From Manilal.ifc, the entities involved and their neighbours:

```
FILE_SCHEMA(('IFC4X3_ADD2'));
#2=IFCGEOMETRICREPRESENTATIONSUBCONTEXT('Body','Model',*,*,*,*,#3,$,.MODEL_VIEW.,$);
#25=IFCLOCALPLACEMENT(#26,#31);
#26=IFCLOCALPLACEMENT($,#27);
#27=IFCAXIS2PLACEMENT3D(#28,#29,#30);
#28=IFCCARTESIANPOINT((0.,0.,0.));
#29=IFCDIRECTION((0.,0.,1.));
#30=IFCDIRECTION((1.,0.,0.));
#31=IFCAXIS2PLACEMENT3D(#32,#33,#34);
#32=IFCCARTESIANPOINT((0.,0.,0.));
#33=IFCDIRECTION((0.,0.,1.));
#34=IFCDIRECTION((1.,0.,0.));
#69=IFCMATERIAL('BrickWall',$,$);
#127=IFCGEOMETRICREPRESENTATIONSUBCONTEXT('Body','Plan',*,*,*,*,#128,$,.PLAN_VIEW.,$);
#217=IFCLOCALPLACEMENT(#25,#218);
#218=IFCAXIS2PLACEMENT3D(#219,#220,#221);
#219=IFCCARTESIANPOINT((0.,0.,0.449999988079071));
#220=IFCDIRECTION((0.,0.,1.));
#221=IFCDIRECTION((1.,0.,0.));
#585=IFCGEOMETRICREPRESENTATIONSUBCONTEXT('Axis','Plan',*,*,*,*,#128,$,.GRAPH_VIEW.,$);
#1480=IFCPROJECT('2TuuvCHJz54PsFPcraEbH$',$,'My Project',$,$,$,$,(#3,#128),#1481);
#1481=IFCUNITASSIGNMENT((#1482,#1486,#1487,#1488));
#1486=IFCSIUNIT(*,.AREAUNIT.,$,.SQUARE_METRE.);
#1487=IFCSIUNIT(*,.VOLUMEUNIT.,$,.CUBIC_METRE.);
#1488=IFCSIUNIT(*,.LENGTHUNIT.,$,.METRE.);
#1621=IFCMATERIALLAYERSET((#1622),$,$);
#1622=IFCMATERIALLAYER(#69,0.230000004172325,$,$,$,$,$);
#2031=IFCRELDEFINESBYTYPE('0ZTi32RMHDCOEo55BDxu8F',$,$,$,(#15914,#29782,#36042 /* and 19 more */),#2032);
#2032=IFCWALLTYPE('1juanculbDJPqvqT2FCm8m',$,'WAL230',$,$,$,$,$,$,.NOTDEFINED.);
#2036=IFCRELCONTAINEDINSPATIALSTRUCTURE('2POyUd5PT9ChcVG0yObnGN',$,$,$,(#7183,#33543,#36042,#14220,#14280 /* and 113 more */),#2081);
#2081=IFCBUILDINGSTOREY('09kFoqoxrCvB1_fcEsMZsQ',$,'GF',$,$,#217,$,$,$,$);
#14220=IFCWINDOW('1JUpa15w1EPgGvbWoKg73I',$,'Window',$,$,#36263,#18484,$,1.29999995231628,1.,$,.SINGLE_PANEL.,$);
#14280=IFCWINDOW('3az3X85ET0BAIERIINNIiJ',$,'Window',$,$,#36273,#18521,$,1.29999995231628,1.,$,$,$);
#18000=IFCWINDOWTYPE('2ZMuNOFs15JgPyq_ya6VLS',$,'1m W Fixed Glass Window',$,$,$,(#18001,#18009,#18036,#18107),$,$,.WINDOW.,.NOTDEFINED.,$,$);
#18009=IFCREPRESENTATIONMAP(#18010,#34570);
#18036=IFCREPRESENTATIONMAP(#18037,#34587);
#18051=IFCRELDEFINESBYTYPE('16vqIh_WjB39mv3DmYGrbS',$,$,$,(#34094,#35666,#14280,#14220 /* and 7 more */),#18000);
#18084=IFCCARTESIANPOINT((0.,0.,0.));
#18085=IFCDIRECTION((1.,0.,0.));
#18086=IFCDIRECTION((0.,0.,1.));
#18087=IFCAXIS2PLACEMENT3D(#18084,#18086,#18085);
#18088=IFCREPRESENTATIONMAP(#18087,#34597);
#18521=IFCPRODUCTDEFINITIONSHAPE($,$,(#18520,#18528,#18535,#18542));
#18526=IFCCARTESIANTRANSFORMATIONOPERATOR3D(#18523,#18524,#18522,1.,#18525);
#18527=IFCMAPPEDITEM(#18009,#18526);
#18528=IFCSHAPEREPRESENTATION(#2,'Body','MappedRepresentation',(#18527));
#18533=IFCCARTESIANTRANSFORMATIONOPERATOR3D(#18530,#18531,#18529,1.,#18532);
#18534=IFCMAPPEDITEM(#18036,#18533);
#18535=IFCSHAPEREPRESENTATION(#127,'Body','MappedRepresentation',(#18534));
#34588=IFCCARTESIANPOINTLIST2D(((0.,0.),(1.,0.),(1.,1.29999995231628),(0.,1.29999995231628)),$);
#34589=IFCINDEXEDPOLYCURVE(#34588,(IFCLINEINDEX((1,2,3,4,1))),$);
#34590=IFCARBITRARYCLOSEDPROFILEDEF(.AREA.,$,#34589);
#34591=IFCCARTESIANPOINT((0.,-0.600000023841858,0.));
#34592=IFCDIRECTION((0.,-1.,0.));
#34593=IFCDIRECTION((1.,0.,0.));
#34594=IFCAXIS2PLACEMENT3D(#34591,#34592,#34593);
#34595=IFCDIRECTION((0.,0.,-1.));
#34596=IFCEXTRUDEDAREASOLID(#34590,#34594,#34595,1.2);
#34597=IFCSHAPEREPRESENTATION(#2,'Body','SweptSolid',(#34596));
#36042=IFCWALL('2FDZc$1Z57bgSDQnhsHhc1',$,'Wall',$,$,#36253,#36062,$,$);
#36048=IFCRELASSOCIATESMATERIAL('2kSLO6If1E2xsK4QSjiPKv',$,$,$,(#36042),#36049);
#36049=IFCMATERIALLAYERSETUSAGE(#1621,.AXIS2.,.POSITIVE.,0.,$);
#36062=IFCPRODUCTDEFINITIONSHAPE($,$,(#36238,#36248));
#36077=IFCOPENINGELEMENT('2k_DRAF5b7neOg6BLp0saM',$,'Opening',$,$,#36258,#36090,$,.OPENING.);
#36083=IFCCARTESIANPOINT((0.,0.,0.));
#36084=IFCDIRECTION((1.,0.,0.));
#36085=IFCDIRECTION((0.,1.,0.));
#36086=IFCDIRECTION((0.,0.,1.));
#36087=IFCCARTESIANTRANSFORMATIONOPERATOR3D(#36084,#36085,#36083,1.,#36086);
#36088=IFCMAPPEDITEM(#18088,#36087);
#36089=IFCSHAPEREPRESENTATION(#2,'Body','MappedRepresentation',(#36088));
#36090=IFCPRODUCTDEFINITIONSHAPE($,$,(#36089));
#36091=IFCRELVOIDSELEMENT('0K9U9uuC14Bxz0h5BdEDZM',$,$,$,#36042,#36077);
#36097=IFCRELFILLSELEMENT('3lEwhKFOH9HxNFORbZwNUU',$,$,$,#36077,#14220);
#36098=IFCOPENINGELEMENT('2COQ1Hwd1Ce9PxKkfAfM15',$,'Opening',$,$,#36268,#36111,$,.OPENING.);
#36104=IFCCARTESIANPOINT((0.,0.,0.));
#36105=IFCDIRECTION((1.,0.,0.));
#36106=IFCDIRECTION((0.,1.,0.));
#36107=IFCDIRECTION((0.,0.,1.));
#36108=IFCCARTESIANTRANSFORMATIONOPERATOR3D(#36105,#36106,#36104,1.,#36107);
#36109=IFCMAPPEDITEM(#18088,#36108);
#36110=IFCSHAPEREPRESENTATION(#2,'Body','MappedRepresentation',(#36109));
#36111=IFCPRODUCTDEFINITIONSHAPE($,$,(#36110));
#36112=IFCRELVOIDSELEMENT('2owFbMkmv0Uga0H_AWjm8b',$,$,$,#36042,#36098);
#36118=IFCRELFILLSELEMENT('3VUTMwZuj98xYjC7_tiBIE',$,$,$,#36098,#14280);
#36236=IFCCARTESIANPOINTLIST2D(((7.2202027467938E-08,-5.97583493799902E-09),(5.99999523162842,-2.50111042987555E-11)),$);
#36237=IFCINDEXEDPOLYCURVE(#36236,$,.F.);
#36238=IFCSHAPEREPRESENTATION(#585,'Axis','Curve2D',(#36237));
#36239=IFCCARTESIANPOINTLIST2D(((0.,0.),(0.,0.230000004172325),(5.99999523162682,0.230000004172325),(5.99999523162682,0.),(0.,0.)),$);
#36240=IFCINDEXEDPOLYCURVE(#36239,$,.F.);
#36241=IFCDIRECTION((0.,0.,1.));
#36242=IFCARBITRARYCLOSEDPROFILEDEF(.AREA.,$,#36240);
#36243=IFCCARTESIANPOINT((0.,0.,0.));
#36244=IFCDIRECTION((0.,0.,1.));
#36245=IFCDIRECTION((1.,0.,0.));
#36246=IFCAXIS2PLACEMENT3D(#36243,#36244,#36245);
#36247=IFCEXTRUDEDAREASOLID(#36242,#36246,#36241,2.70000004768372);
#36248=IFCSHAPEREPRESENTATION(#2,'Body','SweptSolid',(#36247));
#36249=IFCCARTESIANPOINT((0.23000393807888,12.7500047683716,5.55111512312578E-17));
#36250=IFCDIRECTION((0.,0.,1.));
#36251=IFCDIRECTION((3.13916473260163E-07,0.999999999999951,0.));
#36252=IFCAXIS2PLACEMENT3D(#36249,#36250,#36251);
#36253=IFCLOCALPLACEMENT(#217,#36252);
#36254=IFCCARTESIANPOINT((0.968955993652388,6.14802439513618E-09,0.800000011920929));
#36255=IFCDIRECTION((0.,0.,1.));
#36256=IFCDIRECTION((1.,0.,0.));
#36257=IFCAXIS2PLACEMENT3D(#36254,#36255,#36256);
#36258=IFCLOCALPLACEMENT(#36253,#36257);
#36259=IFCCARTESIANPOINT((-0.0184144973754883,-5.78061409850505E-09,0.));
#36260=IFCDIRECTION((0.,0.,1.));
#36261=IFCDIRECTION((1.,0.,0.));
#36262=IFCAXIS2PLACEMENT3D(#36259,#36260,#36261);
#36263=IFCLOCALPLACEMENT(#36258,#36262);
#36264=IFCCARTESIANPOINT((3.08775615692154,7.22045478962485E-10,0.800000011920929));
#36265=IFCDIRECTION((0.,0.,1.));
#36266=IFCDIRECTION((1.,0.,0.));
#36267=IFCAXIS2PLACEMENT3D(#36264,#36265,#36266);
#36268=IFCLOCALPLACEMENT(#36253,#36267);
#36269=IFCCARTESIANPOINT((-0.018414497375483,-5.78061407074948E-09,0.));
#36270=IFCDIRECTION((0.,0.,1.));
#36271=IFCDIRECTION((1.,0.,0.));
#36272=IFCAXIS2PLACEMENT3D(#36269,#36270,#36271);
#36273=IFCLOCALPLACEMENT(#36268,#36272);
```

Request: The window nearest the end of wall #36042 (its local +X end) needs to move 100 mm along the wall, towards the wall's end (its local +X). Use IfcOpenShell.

```python
import ifcopenshell
import ifcopenshell.api.geometry
import ifcopenshell.util.placement
import ifcopenshell.util.unit

model = ifcopenshell.open("Manilal.ifc")
unit_scale = ifcopenshell.util.unit.calculate_unit_scale(model)

window = model.by_guid("3az3X85ET0BAIERIINNIiJ")
opening = window.FillsVoids[0].RelatingOpeningElement
wall = opening.VoidsElements[0].RelatingBuildingElement

wall_matrix = ifcopenshell.util.placement.get_local_placement(wall.ObjectPlacement)
shift = wall_matrix[:3, 0] * 0.1 / unit_scale
before = ifcopenshell.util.placement.get_local_placement(window.ObjectPlacement)[:3, 3].copy()

# The window is placed relative to its opening, so it follows when the opening moves.
matrix = ifcopenshell.util.placement.get_local_placement(opening.ObjectPlacement)
matrix[:3, 3] += shift
ifcopenshell.api.geometry.edit_object_placement(
    model, product=opening, matrix=matrix, is_si=False, should_transform_children=True
)

after = ifcopenshell.util.placement.get_local_placement(window.ObjectPlacement)[:3, 3]
print("window moved by", (after - before).round(3) + 0.0)

model.write("Manilal-out.ifc")
```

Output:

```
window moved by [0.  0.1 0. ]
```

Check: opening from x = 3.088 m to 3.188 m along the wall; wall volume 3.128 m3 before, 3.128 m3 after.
